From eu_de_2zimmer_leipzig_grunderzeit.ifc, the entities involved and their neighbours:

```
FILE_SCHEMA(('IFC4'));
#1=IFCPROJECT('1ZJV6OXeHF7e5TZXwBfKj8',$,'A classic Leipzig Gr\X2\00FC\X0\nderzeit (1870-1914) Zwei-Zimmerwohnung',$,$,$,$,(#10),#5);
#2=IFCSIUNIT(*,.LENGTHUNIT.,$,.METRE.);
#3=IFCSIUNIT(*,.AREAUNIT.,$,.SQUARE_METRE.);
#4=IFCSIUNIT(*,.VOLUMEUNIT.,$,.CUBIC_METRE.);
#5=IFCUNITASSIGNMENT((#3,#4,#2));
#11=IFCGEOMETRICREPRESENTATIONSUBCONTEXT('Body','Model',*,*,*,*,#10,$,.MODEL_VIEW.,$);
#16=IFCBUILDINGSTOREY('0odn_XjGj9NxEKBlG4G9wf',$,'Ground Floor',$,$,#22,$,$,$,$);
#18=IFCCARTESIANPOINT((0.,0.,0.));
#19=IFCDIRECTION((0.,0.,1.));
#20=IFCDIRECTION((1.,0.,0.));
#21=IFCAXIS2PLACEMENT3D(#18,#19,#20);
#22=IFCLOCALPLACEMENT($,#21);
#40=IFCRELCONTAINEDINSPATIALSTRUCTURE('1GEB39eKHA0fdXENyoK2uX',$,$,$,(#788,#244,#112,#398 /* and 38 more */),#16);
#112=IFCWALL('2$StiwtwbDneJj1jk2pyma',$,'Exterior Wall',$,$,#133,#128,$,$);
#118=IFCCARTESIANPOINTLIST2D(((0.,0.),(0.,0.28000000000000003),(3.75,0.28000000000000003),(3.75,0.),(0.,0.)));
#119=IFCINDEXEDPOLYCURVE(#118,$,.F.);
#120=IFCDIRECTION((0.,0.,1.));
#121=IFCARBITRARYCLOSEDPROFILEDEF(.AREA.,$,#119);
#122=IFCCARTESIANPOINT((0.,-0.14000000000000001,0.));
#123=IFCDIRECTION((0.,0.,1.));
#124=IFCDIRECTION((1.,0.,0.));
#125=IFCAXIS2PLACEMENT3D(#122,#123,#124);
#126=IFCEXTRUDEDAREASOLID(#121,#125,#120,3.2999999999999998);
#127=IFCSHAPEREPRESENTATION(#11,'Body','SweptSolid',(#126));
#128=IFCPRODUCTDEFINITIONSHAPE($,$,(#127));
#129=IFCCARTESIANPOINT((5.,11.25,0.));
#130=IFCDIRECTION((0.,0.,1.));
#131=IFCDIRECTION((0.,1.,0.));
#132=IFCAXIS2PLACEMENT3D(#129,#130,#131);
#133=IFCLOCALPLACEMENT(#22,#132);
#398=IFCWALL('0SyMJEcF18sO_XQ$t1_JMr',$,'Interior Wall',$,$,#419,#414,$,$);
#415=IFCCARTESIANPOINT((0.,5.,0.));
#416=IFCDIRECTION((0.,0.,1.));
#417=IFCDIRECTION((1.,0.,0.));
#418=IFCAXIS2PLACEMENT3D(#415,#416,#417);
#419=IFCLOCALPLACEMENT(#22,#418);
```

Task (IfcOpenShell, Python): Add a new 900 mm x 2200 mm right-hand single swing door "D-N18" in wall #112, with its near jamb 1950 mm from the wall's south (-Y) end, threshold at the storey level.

```python
import numpy as np
import ifcopenshell
import ifcopenshell.api.feature
import ifcopenshell.api.geometry
import ifcopenshell.api.root
import ifcopenshell.api.spatial
import ifcopenshell.geom
import ifcopenshell.util.element
import ifcopenshell.util.placement
import ifcopenshell.util.representation
import ifcopenshell.util.shape
import ifcopenshell.util.unit

model = ifcopenshell.open("eu_de_2zimmer_leipzig_grunderzeit.ifc")
unit_scale = ifcopenshell.util.unit.calculate_unit_scale(model)
settings = ifcopenshell.geom.settings()


def volume(element):
    """Net volume in cubic metres, openings subtracted."""
    shape = ifcopenshell.geom.create_shape(settings, element)
    return ifcopenshell.util.shape.get_volume(shape.geometry)


wall = model.by_guid("2$StiwtwbDneJj1jk2pyma")
storey = ifcopenshell.util.element.get_container(wall, ifc_class="IfcBuildingStorey")
context = ifcopenshell.util.representation.get_context(model, "Model", "Body", "MODEL_VIEW")
before = volume(wall)

width, height, from_end, sill = 0.9, 2.2, 1.95, 0.0  # metres

# The wall runs along its own X axis, and the end named is its -X end.
wall_shape = ifcopenshell.geom.create_shape(settings, wall)
x, y, z = ifcopenshell.util.shape.get_vertices(wall_shape.geometry).T
start = x.min() + from_end
face, thickness = float(y.min()), float(y.max() - y.min())
wall_matrix = ifcopenshell.util.placement.get_local_placement(wall.ObjectPlacement)
level = ifcopenshell.util.placement.get_local_placement(storey.ObjectPlacement)[2, 3]


def in_wall(x, y):
    """Placement at x, y metres in the wall's axes, at sill height."""
    matrix = wall_matrix.copy()
    matrix[:, 3] = wall_matrix @ np.array([x / unit_scale, y / unit_scale, 0.0, 1.0])
    matrix[2, 3] = level + sill / unit_scale
    return matrix


# Opening: a box that overshoots both wall faces by 50 mm.
opening = ifcopenshell.api.root.create_entity(model, ifc_class="IfcOpeningElement", predefined_type="OPENING")
box = ifcopenshell.api.geometry.add_wall_representation(
    model, context=context, length=width, height=height, thickness=thickness + 0.1
)
ifcopenshell.api.geometry.assign_representation(model, product=opening, representation=box)
ifcopenshell.api.geometry.edit_object_placement(model, product=opening, matrix=in_wall(start, face - 0.05), is_si=False)
ifcopenshell.api.feature.add_feature(model, feature=opening, element=wall)

door = ifcopenshell.api.root.create_entity(model, ifc_class="IfcDoor", name="D-N18", predefined_type="DOOR")
door.OverallWidth, door.OverallHeight = width / unit_scale, height / unit_scale
door.OperationType = "SINGLE_SWING_RIGHT"
body = ifcopenshell.api.geometry.add_door_representation(
    model,
    context=context,
    overall_width=door.OverallWidth,
    overall_height=door.OverallHeight,
    operation_type="SINGLE_SWING_RIGHT",
    lining_properties={"LiningDepth": thickness / unit_scale, "ThresholdDepth": thickness / unit_scale},
)
ifcopenshell.api.geometry.assign_representation(model, product=door, representation=body)
ifcopenshell.api.spatial.assign_container(model, products=[door], relating_structure=storey)
ifcopenshell.api.feature.add_filling(model, opening=opening, element=door)

# The lining spans the wall, so the door starts at the wall face.
ifcopenshell.api.geometry.edit_object_placement(model, product=door, matrix=in_wall(start, face), is_si=False)

after = volume(wall)

print(f"wall volume {before:.3f} -> {after:.3f} m3")

model.write("eu_de_2zimmer_leipzig_grunderzeit_edited.ifc")
```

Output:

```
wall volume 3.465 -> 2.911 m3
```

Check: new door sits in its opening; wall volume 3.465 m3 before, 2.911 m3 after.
